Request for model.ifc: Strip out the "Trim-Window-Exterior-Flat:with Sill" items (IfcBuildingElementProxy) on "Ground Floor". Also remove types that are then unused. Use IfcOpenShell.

First a look at what the model holds.

```python
import ifcopenshell
import ifcopenshell.util.element

model = ifcopenshell.open("model.ifc")
print(model.schema)
storey = next(s for s in model.by_type("IfcBuildingStorey") if s.Name == "Ground Floor")
proxies = [e for e in ifcopenshell.util.element.get_decomposition(storey) if e.is_a("IfcBuildingElementProxy")]
seen = {}
for e in proxies:
    element_type = ifcopenshell.util.element.get_type(e)
    name = element_type.Name if element_type not in (None, e) else None
    seen[name] = seen.get(name, 0) + 1
for name, count in sorted(seen.items(), key=str):
    print(count, "x", name)
```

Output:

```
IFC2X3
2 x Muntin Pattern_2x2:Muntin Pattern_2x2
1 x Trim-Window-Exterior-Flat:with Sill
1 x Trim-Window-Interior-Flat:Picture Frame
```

```python
import ifcopenshell
import ifcopenshell.api.root
import ifcopenshell.util.element

model = ifcopenshell.open("model.ifc")

storey = next(s for s in model.by_type("IfcBuildingStorey") if s.Name == "Ground Floor")
proxies = [e for e in ifcopenshell.util.element.get_decomposition(storey) if e.is_a("IfcBuildingElementProxy")]
targets = [e for e in proxies if (t := ifcopenshell.util.element.get_type(e)) not in (None, e) and t.Name == "Trim-Window-Exterior-Flat:with Sill"]
types = {ifcopenshell.util.element.get_type(e) for e in targets} - {None, *targets}

for e in targets:
    ifcopenshell.api.root.remove_product(model, product=e)
print(len(targets), "removed")

unused = [t for t in types if not ifcopenshell.util.element.get_types(t)]
for t in unused:
    ifcopenshell.api.root.remove_product(model, product=t)
print(len(unused), "unused types removed")

model.write("model_updated.ifc")
```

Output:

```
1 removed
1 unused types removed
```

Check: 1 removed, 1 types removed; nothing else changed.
